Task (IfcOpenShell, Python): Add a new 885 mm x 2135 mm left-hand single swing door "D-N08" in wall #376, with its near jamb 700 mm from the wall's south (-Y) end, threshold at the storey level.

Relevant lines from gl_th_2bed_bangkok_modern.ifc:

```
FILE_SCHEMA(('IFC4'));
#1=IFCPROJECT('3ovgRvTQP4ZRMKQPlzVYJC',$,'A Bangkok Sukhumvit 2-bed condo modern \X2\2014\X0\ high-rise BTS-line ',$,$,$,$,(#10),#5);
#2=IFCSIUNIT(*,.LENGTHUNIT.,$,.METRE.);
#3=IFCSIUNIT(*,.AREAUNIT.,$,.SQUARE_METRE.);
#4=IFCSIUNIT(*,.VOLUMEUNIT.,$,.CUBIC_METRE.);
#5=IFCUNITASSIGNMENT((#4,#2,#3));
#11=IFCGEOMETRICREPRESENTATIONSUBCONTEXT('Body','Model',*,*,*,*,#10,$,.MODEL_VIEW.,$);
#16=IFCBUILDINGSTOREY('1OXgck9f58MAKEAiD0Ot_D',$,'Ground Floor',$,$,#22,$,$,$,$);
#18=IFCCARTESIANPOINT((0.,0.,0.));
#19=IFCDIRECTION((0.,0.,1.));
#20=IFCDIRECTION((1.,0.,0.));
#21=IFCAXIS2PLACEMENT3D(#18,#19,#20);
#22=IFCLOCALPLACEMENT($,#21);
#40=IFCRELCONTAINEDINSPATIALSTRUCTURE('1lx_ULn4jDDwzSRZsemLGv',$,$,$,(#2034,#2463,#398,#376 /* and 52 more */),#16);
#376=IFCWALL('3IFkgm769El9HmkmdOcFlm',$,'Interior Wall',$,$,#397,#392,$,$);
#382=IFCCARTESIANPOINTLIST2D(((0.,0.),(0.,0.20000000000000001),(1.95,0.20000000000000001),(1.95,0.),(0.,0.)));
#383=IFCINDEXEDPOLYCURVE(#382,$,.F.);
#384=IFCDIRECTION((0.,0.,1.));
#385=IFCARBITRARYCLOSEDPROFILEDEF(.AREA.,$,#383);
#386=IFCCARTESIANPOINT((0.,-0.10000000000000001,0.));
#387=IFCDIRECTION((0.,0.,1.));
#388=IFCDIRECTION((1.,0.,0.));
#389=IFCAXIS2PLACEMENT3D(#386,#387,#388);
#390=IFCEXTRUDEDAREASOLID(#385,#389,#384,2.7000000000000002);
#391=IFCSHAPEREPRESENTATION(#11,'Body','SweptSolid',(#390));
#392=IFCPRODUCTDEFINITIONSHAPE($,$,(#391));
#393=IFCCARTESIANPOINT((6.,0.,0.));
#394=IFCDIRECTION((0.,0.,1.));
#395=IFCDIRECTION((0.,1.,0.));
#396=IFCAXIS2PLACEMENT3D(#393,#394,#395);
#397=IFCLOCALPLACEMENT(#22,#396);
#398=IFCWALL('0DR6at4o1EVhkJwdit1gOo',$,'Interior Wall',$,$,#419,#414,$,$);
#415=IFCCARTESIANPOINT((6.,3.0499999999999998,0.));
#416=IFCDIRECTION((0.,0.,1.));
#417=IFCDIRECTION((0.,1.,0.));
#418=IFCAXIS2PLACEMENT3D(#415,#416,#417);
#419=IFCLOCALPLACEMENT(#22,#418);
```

```python
import numpy as np
import ifcopenshell
import ifcopenshell.api.feature
import ifcopenshell.api.geometry
import ifcopenshell.api.root
import ifcopenshell.api.spatial
import ifcopenshell.geom
import ifcopenshell.util.element
import ifcopenshell.util.placement
import ifcopenshell.util.representation
import ifcopenshell.util.shape
import ifcopenshell.util.unit

model = ifcopenshell.open("gl_th_2bed_bangkok_modern.ifc")
unit_scale = ifcopenshell.util.unit.calculate_unit_scale(model)
settings = ifcopenshell.geom.settings()


def volume(element):
    """Net volume in cubic metres, openings subtracted."""
    shape = ifcopenshell.geom.create_shape(settings, element)
    return ifcopenshell.util.shape.get_volume(shape.geometry)


wall = model.by_guid("3IFkgm769El9HmkmdOcFlm")
storey = ifcopenshell.util.element.get_container(wall, ifc_class="IfcBuildingStorey")
context = ifcopenshell.util.representation.get_context(model, "Model", "Body", "MODEL_VIEW")
before = volume(wall)

width, height, from_end, sill = 0.885, 2.135, 0.7, 0.0  # metres

# The wall runs along its own X axis, and the end named is its -X end.
wall_shape = ifcopenshell.geom.create_shape(settings, wall)
x, y, z = ifcopenshell.util.shape.get_vertices(wall_shape.geometry).T
start = x.min() + from_end
face, thickness = float(y.min()), float(y.max() - y.min())
wall_matrix = ifcopenshell.util.placement.get_local_placement(wall.ObjectPlacement)
level = ifcopenshell.util.placement.get_local_placement(storey.ObjectPlacement)[2, 3]


def in_wall(x, y):
    """Placement at x, y metres in the wall's axes, at sill height."""
    matrix = wall_matrix.copy()
    matrix[:, 3] = wall_matrix @ np.array([x / unit_scale, y / unit_scale, 0.0, 1.0])
    matrix[2, 3] = level + sill / unit_scale
    return matrix


# Opening: a box that overshoots both wall faces by 50 mm.
opening = ifcopenshell.api.root.create_entity(model, ifc_class="IfcOpeningElement", predefined_type="OPENING")
box = ifcopenshell.api.geometry.add_wall_representation(
    model, context=context, length=width, height=height, thickness=thickness + 0.1
)
ifcopenshell.api.geometry.assign_representation(model, product=opening, representation=box)
ifcopenshell.api.geometry.edit_object_placement(model, product=opening, matrix=in_wall(start, face - 0.05), is_si=False)
ifcopenshell.api.feature.add_feature(model, feature=opening, element=wall)

door = ifcopenshell.api.root.create_entity(model, ifc_class="IfcDoor", name="D-N08", predefined_type="DOOR")
door.OverallWidth, door.OverallHeight = width / unit_scale, height / unit_scale
door.OperationType = "SINGLE_SWING_LEFT"
body = ifcopenshell.api.geometry.add_door_representation(
    model,
    context=context,
    overall_width=door.OverallWidth,
    overall_height=door.OverallHeight,
    operation_type="SINGLE_SWING_LEFT",
    lining_properties={"LiningDepth": thickness / unit_scale, "ThresholdDepth": thickness / unit_scale},
)
ifcopenshell.api.geometry.assign_representation(model, product=door, representation=body)
ifcopenshell.api.spatial.assign_container(model, products=[door], relating_structure=storey)
ifcopenshell.api.feature.add_filling(model, opening=opening, element=door)

# The lining spans the wall, so the door starts at the wall face.
ifcopenshell.api.geometry.edit_object_placement(model, product=door, matrix=in_wall(start, face), is_si=False)

after = volume(wall)

print(f"wall volume {before:.3f} -> {after:.3f} m3")

model.write("gl_th_2bed_bangkok_modern_rev.ifc")
```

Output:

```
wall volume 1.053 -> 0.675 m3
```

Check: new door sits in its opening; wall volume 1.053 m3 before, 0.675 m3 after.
